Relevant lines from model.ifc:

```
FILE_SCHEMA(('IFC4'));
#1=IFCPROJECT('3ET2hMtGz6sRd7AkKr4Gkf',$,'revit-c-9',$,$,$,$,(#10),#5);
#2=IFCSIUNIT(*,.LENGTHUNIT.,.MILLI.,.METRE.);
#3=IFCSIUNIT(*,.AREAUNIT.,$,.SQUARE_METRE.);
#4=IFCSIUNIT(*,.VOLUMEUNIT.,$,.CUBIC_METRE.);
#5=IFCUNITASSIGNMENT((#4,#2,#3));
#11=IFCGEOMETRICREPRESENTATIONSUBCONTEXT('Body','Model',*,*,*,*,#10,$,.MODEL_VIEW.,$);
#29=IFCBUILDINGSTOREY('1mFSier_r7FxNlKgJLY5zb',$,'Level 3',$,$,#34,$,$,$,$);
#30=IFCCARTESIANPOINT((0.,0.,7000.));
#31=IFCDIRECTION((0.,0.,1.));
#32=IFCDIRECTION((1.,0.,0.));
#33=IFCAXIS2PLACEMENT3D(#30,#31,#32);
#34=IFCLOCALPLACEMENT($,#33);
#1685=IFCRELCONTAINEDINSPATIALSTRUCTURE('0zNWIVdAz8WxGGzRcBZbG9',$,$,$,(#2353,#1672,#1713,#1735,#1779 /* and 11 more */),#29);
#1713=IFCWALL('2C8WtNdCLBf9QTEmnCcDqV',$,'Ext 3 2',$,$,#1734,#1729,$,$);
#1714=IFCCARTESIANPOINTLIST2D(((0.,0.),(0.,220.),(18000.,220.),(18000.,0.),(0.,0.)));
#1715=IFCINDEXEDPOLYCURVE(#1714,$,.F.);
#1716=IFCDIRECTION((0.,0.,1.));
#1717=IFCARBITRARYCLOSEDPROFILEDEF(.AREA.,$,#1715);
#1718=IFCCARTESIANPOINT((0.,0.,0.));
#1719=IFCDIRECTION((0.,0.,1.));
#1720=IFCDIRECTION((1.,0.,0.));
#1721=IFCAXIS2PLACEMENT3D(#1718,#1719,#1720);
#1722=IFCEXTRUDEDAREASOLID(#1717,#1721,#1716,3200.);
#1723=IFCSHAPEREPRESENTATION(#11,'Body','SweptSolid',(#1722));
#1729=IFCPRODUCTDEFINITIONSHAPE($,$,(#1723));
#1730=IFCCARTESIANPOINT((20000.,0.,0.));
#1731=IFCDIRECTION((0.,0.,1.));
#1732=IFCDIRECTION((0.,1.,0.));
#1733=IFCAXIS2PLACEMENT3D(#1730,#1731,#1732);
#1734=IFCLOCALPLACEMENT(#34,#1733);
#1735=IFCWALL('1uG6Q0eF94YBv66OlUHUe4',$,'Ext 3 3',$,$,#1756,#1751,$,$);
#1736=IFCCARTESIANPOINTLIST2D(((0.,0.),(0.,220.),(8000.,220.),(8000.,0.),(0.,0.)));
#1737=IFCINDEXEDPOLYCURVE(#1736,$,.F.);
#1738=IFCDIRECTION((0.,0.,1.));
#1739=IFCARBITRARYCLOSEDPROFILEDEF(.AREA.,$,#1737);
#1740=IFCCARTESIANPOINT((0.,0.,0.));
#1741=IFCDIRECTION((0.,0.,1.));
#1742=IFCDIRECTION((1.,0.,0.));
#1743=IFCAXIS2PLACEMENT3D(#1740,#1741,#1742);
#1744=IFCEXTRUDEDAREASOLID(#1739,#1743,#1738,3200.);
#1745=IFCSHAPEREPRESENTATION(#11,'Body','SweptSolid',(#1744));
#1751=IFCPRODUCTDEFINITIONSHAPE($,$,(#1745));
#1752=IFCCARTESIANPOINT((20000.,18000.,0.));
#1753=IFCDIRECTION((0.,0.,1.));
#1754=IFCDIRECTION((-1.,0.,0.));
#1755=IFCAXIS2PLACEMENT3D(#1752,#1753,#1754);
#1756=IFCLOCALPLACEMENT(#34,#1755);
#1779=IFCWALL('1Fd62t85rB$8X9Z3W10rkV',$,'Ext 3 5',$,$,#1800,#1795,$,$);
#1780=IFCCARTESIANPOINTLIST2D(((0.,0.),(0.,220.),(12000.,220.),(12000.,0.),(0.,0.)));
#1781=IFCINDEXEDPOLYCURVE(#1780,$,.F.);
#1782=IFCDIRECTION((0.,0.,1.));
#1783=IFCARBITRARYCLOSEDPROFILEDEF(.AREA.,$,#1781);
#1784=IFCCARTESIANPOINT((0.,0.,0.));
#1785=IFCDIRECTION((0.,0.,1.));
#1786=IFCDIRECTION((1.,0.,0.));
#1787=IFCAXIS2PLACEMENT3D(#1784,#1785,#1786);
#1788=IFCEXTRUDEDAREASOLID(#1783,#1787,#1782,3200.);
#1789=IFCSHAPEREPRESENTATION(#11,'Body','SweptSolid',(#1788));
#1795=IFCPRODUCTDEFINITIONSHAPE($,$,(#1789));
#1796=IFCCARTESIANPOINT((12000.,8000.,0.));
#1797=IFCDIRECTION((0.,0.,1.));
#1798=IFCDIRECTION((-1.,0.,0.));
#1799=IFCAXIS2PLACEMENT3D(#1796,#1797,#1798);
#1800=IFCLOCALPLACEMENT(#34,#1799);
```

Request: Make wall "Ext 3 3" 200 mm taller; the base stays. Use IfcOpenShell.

```python
import ifcopenshell
import ifcopenshell.geom
import ifcopenshell.util.representation
import ifcopenshell.util.shape
import ifcopenshell.util.unit

model = ifcopenshell.open("model.ifc")
unit_scale = ifcopenshell.util.unit.calculate_unit_scale(model)
settings = ifcopenshell.geom.settings()


def volume(element):
    """Net volume in cubic metres, openings subtracted."""
    shape = ifcopenshell.geom.create_shape(settings, element)
    return ifcopenshell.util.shape.get_volume(shape.geometry)


wall = model.by_guid("1uG6Q0eF94YBv66OlUHUe4")
before = volume(wall)

body = ifcopenshell.util.representation.get_representation(wall, "Model", "Body")
solid = body.Items[0]
old_height = solid.Depth
solid.Depth += 0.2 / unit_scale
after = volume(wall)

print(f"height {old_height:g} -> {solid.Depth:g}, volume {before:.3f} -> {after:.3f} m3")

model.write("model_updated.ifc")
```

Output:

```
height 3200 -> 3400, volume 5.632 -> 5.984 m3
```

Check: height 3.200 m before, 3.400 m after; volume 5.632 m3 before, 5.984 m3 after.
